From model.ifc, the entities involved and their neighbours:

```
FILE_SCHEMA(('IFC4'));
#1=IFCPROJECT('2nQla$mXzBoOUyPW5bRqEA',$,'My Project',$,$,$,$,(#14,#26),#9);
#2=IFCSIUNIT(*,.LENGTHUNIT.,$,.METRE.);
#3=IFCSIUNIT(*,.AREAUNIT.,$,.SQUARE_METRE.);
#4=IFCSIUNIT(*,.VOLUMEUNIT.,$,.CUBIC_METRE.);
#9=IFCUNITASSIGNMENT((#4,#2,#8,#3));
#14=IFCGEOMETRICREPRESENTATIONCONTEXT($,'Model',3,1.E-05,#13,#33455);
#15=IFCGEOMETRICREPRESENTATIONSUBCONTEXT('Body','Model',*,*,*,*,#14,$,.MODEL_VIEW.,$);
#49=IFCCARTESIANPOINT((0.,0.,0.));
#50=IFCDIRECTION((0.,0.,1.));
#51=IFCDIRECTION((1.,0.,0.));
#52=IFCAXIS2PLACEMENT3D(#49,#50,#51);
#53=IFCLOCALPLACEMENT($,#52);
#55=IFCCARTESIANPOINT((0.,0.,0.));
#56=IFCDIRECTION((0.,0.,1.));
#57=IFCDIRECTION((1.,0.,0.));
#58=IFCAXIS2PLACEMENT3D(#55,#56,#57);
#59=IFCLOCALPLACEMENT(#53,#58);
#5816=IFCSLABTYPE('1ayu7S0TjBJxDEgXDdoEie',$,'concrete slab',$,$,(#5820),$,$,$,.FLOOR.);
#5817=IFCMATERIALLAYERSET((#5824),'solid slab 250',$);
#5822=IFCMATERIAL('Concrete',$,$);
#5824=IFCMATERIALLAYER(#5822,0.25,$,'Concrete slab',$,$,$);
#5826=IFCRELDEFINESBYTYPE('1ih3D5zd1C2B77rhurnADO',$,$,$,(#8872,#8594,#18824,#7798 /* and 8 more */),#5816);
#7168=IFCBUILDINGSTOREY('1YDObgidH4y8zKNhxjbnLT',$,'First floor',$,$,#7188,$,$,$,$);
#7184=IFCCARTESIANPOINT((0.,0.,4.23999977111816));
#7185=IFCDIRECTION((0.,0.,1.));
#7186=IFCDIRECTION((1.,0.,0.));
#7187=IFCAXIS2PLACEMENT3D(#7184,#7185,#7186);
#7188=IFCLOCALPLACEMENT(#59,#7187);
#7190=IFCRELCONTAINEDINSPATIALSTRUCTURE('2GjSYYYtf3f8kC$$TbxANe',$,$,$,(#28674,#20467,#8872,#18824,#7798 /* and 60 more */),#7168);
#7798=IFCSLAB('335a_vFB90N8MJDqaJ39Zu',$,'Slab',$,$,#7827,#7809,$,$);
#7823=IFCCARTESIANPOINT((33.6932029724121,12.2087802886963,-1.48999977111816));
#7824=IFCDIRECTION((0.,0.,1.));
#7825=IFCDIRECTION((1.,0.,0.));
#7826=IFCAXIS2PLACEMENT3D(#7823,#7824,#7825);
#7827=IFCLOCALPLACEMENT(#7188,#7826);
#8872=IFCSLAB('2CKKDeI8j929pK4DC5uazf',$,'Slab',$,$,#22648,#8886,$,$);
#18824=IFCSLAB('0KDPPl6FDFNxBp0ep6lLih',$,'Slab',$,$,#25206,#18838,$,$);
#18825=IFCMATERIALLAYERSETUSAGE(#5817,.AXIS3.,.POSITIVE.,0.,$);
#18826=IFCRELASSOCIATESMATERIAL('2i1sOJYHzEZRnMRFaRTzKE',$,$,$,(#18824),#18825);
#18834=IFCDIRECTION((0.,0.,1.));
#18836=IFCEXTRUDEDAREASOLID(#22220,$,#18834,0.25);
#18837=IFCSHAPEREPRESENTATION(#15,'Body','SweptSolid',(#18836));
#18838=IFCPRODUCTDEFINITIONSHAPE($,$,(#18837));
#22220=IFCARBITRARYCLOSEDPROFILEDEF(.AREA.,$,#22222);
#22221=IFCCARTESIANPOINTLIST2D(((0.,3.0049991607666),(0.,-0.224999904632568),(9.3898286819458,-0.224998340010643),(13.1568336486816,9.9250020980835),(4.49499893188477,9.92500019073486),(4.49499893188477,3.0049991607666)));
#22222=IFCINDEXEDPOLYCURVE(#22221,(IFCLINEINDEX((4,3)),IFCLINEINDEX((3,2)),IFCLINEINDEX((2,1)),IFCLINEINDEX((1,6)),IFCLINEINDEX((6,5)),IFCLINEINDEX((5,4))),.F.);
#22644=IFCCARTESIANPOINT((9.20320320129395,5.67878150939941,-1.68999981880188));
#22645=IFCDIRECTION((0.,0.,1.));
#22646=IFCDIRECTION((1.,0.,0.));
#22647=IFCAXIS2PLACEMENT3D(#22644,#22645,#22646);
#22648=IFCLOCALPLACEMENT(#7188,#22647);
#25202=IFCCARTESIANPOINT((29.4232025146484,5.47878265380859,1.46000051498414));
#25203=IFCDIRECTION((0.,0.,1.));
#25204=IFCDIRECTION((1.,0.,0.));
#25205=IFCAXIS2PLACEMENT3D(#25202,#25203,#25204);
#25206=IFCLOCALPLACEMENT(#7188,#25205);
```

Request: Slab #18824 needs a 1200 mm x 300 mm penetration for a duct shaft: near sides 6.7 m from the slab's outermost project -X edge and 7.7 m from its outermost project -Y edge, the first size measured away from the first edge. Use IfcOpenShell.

```python
import numpy as np
import ifcopenshell
import ifcopenshell.api.feature
import ifcopenshell.api.geometry
import ifcopenshell.api.root
import ifcopenshell.geom
import ifcopenshell.util.placement
import ifcopenshell.util.representation
import ifcopenshell.util.shape
import ifcopenshell.util.unit

model = ifcopenshell.open("model.ifc")
unit_scale = ifcopenshell.util.unit.calculate_unit_scale(model)
settings = ifcopenshell.geom.settings()


def volume(element):
    """Net volume in cubic metres, openings subtracted."""
    shape = ifcopenshell.geom.create_shape(settings, element)
    return ifcopenshell.util.shape.get_volume(shape.geometry)


slab = model.by_guid("0KDPPl6FDFNxBp0ep6lLih")
before = volume(slab)

# Extent in the slab's own axes, in metres. The edges named are its -X and -Y sides.
slab_shape = ifcopenshell.geom.create_shape(settings, slab)
vertices = ifcopenshell.util.shape.get_vertices(slab_shape.geometry)
x_min, y_min, bottom = vertices.min(axis=0)
top = vertices[:, 2].max()

opening = ifcopenshell.api.root.create_entity(model, ifc_class="IfcOpeningElement", name="Duct shaft opening", predefined_type="OPENING")
context = ifcopenshell.util.representation.get_context(model, "Model", "Body", "MODEL_VIEW")
width, depth = 1.2, 0.3
outline = [(0.0, 0.0), (width, 0.0), (width, depth), (0.0, depth), (0.0, 0.0)]
# Overshoot both faces by 50 mm so the cut is clean.
shape = ifcopenshell.api.geometry.add_slab_representation(
    model, context=context, depth=top - bottom + 0.1, polyline=outline
)
ifcopenshell.api.geometry.assign_representation(model, product=opening, representation=shape)

matrix = ifcopenshell.util.placement.get_local_placement(slab.ObjectPlacement)
matrix[:, 3] = matrix @ np.append(np.array([x_min + 6.7, y_min + 7.7, bottom - 0.05]) / unit_scale, 1.0)
ifcopenshell.api.geometry.edit_object_placement(model, product=opening, matrix=matrix, is_si=False)
ifcopenshell.api.feature.add_feature(model, feature=opening, element=slab)

after = volume(slab)

print(f"slab volume {before:.3f} -> {after:.3f} m3")

model.write("model_rev.ifc")
```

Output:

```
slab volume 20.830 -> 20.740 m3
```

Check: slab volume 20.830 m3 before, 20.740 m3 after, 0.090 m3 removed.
